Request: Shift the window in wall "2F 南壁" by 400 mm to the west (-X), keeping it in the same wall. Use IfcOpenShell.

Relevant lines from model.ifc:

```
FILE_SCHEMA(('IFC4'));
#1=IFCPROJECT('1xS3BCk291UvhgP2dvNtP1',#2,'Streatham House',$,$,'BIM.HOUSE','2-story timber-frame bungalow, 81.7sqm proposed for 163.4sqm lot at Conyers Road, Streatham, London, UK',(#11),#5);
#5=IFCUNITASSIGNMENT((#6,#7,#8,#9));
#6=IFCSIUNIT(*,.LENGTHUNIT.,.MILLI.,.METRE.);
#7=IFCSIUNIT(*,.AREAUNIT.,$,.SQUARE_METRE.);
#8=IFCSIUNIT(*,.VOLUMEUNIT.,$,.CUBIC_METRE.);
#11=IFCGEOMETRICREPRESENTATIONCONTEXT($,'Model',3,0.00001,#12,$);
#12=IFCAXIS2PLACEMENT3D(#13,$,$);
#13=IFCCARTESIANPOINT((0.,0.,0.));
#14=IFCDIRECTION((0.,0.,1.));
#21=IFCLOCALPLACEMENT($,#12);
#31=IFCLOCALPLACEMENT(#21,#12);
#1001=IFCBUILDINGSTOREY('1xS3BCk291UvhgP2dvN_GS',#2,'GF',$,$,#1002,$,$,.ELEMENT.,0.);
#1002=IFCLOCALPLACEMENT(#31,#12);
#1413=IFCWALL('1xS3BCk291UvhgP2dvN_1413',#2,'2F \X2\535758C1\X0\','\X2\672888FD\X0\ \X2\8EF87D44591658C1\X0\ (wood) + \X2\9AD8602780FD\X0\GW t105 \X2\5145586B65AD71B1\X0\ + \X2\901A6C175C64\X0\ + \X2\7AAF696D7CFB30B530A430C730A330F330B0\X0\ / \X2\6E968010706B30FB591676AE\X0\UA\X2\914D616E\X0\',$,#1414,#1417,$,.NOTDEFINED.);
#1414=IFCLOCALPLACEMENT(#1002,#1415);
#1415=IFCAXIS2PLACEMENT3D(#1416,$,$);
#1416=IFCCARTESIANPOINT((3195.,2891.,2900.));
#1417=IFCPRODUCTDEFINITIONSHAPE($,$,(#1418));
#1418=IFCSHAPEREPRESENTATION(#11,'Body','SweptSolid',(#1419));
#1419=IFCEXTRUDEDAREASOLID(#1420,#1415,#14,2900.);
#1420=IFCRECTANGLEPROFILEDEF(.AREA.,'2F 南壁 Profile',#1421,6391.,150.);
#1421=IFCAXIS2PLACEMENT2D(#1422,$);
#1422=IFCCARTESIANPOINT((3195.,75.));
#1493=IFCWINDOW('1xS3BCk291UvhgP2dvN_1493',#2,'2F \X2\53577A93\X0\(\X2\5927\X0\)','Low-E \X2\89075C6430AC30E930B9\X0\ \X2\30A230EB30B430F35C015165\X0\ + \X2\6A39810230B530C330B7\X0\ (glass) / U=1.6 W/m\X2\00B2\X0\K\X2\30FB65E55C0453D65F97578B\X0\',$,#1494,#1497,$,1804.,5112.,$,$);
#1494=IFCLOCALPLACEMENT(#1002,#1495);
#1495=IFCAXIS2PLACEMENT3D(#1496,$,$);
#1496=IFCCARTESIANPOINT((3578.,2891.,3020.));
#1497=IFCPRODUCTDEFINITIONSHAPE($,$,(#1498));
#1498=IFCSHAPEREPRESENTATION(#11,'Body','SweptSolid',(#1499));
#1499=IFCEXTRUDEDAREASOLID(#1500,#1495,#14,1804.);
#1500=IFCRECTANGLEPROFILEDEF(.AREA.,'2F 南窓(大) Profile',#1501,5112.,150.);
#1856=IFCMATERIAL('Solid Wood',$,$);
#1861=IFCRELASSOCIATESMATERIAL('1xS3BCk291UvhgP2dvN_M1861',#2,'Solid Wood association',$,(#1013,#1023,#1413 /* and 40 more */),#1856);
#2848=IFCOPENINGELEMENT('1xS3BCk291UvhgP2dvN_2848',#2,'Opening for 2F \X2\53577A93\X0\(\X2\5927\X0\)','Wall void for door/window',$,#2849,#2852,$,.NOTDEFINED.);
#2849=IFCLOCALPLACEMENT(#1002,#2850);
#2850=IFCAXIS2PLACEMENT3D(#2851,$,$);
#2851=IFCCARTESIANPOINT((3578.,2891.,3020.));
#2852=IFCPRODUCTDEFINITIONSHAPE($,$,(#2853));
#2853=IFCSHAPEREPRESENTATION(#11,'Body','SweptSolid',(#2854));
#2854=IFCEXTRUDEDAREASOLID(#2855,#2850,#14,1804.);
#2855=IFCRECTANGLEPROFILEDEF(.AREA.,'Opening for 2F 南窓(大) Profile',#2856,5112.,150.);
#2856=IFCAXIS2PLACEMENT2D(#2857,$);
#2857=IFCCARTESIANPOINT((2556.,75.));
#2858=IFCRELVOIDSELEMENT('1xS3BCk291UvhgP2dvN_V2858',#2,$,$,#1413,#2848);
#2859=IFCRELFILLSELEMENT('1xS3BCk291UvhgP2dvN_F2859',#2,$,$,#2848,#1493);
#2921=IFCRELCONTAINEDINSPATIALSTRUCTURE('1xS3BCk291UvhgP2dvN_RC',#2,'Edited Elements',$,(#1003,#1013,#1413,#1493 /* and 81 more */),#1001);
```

```python
import ifcopenshell
import ifcopenshell.api.geometry
import ifcopenshell.util.placement
import ifcopenshell.util.unit

model = ifcopenshell.open("model.ifc")
unit_scale = ifcopenshell.util.unit.calculate_unit_scale(model)

window = model.by_id(1493)
opening = window.FillsVoids[0].RelatingOpeningElement
wall = opening.VoidsElements[0].RelatingBuildingElement

wall_matrix = ifcopenshell.util.placement.get_local_placement(wall.ObjectPlacement)
shift = wall_matrix[:3, 0] * -0.4 / unit_scale
before = ifcopenshell.util.placement.get_local_placement(window.ObjectPlacement)[:3, 3].copy()

# The window is not placed relative to its opening, so move both.
for product in (opening, window):
    matrix = ifcopenshell.util.placement.get_local_placement(product.ObjectPlacement)
    matrix[:3, 3] += shift
    ifcopenshell.api.geometry.edit_object_placement(model, product=product, matrix=matrix, is_si=False)

after = ifcopenshell.util.placement.get_local_placement(window.ObjectPlacement)[:3, 3]
print("window moved by", (after - before).round(3) + 0.0)

model.write("model_rev.ifc")
```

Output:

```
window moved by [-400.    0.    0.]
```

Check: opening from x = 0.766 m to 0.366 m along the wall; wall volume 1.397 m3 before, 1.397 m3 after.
